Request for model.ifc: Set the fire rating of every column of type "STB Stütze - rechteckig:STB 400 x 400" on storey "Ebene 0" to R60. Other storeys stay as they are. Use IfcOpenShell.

First a look at what the model holds.

```python
import ifcopenshell
import ifcopenshell.util.element

model = ifcopenshell.open("model.ifc")
print(model.schema)
storey = next(s for s in model.by_type("IfcBuildingStorey") if s.Name == "Ebene 0")
columns = [e for e in ifcopenshell.util.element.get_decomposition(storey) if e.is_a("IfcColumn")]
seen = {}
for e in columns:
    element_type = ifcopenshell.util.element.get_type(e)
    key = (element_type.Name if element_type != e and element_type else None, ifcopenshell.util.element.get_pset(e, "Pset_ColumnCommon", "FireRating"))
    seen[key] = seen.get(key, 0) + 1
for (name, value), count in sorted(seen.items(), key=str):
    print(count, "x", name, "|", value)
```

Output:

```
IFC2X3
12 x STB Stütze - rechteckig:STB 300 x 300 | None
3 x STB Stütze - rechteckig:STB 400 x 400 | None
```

```python
import ifcopenshell
import ifcopenshell.api.pset
import ifcopenshell.util.element

model = ifcopenshell.open("model.ifc")

storey = next(s for s in model.by_type("IfcBuildingStorey") if s.Name == "Ebene 0")
columns = [e for e in ifcopenshell.util.element.get_decomposition(storey) if e.is_a("IfcColumn")]

count = 0
for e in columns:
    element_type = ifcopenshell.util.element.get_type(e)
    if element_type in (None, e) or element_type.Name != "STB Stütze - rechteckig:STB 400 x 400":
        continue
    # add_pset returns the element's existing set when there is one.
    pset = ifcopenshell.api.pset.add_pset(model, product=e, name="Pset_ColumnCommon")
    ifcopenshell.api.pset.edit_pset(model, pset=pset, properties={"FireRating": "R60"})
    count += 1

print(count, "columns updated")

model.write("model-out.ifc")
```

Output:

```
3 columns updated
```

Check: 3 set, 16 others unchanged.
